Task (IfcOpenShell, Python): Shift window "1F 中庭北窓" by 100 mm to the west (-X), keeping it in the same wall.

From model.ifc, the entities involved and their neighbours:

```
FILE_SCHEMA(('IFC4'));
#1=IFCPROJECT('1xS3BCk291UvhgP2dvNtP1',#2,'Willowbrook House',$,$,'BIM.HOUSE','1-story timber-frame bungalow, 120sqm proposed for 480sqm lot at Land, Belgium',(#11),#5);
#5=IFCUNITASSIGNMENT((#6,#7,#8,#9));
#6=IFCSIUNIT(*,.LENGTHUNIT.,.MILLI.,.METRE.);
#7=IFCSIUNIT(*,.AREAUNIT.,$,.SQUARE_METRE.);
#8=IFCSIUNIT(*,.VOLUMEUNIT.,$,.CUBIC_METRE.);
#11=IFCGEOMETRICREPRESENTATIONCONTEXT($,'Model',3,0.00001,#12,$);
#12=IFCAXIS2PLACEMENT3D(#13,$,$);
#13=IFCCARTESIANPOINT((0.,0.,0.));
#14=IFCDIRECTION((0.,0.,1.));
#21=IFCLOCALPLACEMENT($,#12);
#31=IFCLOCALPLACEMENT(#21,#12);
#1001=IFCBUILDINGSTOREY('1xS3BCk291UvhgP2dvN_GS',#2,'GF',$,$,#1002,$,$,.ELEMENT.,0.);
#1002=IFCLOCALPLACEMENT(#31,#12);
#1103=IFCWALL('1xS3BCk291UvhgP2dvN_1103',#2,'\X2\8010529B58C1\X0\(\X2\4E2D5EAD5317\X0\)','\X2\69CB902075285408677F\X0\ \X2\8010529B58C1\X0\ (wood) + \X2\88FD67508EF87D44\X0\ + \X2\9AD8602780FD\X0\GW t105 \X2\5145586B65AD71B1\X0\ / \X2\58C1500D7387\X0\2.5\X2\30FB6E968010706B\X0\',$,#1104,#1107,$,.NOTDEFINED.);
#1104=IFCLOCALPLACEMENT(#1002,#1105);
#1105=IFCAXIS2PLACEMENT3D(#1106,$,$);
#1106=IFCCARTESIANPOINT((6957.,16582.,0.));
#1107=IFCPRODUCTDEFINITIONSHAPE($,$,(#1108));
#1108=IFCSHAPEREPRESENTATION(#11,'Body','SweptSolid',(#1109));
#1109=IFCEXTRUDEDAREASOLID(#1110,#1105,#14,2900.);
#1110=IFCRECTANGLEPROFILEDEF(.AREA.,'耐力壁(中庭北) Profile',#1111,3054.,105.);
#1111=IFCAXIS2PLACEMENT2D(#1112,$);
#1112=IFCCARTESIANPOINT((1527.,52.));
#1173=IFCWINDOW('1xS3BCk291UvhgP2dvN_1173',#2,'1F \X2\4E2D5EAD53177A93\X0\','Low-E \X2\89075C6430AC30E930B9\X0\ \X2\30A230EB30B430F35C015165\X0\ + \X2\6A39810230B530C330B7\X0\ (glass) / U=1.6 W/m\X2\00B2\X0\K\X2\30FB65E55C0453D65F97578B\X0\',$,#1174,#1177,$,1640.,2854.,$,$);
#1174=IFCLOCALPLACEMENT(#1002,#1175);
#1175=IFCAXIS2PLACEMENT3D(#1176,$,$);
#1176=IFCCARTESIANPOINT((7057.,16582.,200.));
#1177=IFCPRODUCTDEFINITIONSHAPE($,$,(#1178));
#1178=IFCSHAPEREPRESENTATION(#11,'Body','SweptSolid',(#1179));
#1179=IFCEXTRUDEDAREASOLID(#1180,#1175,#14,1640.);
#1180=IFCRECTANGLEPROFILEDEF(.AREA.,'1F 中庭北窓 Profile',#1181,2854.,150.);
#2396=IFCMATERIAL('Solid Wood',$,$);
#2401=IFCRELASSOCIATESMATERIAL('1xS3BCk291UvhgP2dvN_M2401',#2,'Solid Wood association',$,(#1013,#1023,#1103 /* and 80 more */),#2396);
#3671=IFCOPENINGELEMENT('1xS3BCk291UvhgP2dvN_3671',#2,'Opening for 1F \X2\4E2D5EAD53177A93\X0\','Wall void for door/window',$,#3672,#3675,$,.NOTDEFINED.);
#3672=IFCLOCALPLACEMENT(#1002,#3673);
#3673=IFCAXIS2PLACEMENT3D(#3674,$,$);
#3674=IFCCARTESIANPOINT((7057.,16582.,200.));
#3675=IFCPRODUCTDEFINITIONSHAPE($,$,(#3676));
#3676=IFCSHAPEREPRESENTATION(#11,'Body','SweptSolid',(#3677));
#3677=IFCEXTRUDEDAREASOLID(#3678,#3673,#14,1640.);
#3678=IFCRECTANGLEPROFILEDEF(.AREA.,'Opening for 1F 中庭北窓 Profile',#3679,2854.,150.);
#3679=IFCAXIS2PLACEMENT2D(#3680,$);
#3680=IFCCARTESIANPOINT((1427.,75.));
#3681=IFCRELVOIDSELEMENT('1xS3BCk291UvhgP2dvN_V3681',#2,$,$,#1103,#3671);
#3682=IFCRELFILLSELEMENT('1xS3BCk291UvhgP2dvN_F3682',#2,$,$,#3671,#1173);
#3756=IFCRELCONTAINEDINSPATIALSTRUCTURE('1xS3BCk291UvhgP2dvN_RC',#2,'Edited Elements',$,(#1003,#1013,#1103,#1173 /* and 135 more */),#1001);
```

```python
import ifcopenshell
import ifcopenshell.api.geometry
import ifcopenshell.util.placement

model = ifcopenshell.open("model.ifc")

window = model.by_id(1173)
opening = window.FillsVoids[0].RelatingOpeningElement
wall = opening.VoidsElements[0].RelatingBuildingElement

wall_matrix = ifcopenshell.util.placement.get_local_placement(wall.ObjectPlacement)
shift = wall_matrix[:3, 0] * -100.0
before = ifcopenshell.util.placement.get_local_placement(window.ObjectPlacement)[:3, 3].copy()

# The window is not placed relative to its opening, so move both.
for product in (opening, window):
    matrix = ifcopenshell.util.placement.get_local_placement(product.ObjectPlacement)
    matrix[:3, 3] += shift
    ifcopenshell.api.geometry.edit_object_placement(model, product=product, matrix=matrix, is_si=False)

after = ifcopenshell.util.placement.get_local_placement(window.ObjectPlacement)[:3, 3]
print("window moved by", (after - before).round(3) + 0.0)

model.write("model_rev.ifc")
```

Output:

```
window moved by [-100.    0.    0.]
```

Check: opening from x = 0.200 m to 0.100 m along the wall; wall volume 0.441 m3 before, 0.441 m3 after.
